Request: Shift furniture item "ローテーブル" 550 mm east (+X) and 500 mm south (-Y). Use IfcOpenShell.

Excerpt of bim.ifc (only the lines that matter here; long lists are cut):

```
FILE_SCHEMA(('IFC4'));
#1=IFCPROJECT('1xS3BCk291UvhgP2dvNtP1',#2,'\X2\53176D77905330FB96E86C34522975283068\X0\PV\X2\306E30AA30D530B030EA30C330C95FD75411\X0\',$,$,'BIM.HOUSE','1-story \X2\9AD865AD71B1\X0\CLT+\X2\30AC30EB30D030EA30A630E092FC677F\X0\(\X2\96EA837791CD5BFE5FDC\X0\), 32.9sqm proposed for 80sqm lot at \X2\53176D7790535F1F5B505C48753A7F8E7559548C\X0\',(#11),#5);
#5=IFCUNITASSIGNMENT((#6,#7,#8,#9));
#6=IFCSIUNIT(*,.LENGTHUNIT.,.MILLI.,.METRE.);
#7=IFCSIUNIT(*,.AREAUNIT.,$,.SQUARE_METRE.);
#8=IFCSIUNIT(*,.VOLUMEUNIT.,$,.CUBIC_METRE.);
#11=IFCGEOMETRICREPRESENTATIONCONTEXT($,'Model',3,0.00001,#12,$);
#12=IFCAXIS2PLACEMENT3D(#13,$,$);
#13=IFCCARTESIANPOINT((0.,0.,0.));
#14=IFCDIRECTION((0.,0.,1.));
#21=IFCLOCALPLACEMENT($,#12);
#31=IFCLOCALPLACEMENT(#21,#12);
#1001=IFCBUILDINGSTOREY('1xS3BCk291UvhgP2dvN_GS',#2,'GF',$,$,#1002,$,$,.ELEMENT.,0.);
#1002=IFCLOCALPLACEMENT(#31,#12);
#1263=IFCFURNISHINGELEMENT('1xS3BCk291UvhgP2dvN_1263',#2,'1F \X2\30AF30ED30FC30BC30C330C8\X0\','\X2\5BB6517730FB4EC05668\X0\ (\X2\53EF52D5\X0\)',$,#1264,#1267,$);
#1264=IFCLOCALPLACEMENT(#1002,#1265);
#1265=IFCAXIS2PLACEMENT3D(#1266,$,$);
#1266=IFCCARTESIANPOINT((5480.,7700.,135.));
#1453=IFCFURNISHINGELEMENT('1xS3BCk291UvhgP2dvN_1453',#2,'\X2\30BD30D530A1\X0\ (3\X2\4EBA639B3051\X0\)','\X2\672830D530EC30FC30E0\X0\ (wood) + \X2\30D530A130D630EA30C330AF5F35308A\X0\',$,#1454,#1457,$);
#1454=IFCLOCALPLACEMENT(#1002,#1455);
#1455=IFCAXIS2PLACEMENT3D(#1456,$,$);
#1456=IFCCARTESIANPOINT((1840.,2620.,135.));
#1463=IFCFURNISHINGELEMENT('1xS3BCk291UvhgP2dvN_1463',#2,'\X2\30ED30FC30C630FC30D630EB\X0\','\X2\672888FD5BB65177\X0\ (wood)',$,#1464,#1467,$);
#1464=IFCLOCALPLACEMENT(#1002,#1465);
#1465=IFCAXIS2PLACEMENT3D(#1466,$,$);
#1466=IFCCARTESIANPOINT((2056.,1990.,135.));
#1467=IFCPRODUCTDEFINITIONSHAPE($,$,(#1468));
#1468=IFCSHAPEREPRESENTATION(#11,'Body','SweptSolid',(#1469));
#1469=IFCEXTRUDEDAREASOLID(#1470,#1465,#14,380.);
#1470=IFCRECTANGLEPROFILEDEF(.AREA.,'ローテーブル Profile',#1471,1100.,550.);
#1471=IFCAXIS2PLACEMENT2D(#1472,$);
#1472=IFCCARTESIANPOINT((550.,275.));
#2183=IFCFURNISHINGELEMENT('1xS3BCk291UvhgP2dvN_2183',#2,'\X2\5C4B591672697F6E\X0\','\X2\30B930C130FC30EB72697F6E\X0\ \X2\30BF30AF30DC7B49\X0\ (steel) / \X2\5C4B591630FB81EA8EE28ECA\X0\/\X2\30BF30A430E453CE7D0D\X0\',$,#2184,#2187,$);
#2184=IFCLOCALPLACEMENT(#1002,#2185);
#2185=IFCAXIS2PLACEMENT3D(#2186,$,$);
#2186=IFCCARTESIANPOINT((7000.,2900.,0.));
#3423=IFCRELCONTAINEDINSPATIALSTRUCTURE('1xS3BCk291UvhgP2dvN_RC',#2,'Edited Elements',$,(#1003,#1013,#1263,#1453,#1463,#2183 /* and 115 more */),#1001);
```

```python
import ifcopenshell
import ifcopenshell.api.geometry
import ifcopenshell.util.placement
import ifcopenshell.util.unit

model = ifcopenshell.open("bim.ifc")
unit_scale = ifcopenshell.util.unit.calculate_unit_scale(model)

item = model.by_guid("1xS3BCk291UvhgP2dvN_1463")
matrix = ifcopenshell.util.placement.get_local_placement(item.ObjectPlacement)
matrix[0, 3] += 0.55 / unit_scale
matrix[1, 3] -= 0.5 / unit_scale
ifcopenshell.api.geometry.edit_object_placement(model, product=item, matrix=matrix, is_si=False)

print(ifcopenshell.util.placement.get_local_placement(item.ObjectPlacement).round(3) + 0.0)

model.write("bim_rev.ifc")
```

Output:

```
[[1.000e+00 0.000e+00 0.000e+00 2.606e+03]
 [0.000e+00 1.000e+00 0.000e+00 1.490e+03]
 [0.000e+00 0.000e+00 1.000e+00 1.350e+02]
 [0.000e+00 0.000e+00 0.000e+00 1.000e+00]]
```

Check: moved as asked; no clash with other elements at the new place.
